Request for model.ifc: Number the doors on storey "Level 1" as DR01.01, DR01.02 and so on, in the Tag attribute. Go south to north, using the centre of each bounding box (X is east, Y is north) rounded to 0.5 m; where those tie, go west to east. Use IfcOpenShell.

First a look at what the model holds.

```python
import ifcopenshell
import ifcopenshell.util.element
import ifcopenshell.util.placement

model = ifcopenshell.open("model.ifc")
print(model.schema)
storey = next(s for s in model.by_type("IfcBuildingStorey") if s.Name == "Level 1")
doors = [e for e in ifcopenshell.util.element.get_decomposition(storey) if e.is_a("IfcDoor")]
for e in sorted(doors, key=lambda e: e.id()):
    origin = ifcopenshell.util.placement.get_local_placement(e.ObjectPlacement)[:3, 3]
    print(e.id(), e.Tag, e.Name, origin.round(2) + 0.0, sep=" | ")
```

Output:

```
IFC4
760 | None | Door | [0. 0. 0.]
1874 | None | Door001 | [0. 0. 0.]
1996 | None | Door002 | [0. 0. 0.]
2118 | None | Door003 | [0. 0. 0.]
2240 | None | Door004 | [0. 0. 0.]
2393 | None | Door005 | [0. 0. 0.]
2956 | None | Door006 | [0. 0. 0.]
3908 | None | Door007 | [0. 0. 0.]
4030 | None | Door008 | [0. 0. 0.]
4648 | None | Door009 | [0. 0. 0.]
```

```python
import ifcopenshell
import ifcopenshell.geom
import ifcopenshell.util.element
import ifcopenshell.util.shape

model = ifcopenshell.open("model.ifc")
settings = ifcopenshell.geom.settings()
settings.set("use-world-coords", True)


def centre(element):
    shape = ifcopenshell.geom.create_shape(settings, element)
    return ifcopenshell.util.shape.get_bbox_centroid(shape.geometry)


storey = next(s for s in model.by_type("IfcBuildingStorey") if s.Name == "Level 1")
doors = [e for e in ifcopenshell.util.element.get_decomposition(storey) if e.is_a("IfcDoor")]

# Insertion points can sit at a corner or the storey origin, so sort by the geometry (in metres).
centres = {e: centre(e) for e in doors}
doors.sort(key=lambda e: (round(centres[e][1] / 0.5), centres[e][0]))

for i, e in enumerate(doors, start=1):
    number = f"DR01.{i:02d}"
    e.Tag = number
    print(e.id(), number)

model.write("model_v2.ifc")
```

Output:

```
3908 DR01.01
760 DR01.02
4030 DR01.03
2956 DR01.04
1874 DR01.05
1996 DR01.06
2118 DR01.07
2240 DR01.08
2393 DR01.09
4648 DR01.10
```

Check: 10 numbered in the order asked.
